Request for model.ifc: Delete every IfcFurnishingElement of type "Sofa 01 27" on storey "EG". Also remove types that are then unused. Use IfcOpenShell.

First a look at what the model holds.

```python
import ifcopenshell
import ifcopenshell.util.element

model = ifcopenshell.open("model.ifc")
print(model.schema)
storey = next(s for s in model.by_type("IfcBuildingStorey") if s.Name == "EG")
furniture = [e for e in ifcopenshell.util.element.get_decomposition(storey) if e.is_a("IfcFurnishingElement")]
seen = {}
for e in furniture:
    element_type = ifcopenshell.util.element.get_type(e)
    name = element_type.Name if element_type not in (None, e) else None
    seen[name] = seen.get(name, 0) + 1
for name, count in sorted(seen.items(), key=str):
    print(count, "x", name)
```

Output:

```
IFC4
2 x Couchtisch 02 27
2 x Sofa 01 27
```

```python
import ifcopenshell
import ifcopenshell.api.root
import ifcopenshell.util.element

model = ifcopenshell.open("model.ifc")

storey = next(s for s in model.by_type("IfcBuildingStorey") if s.Name == "EG")
furniture = [e for e in ifcopenshell.util.element.get_decomposition(storey) if e.is_a("IfcFurnishingElement")]
targets = [e for e in furniture if (t := ifcopenshell.util.element.get_type(e)) not in (None, e) and t.Name == "Sofa 01 27"]
types = {ifcopenshell.util.element.get_type(e) for e in targets} - {None, *targets}

for e in targets:
    ifcopenshell.api.root.remove_product(model, product=e)
print(len(targets), "removed")

unused = [t for t in types if not ifcopenshell.util.element.get_types(t)]
for t in unused:
    ifcopenshell.api.root.remove_product(model, product=t)
print(len(unused), "unused types removed")

model.write("model_v2.ifc")
```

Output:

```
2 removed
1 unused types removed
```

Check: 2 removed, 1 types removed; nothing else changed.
